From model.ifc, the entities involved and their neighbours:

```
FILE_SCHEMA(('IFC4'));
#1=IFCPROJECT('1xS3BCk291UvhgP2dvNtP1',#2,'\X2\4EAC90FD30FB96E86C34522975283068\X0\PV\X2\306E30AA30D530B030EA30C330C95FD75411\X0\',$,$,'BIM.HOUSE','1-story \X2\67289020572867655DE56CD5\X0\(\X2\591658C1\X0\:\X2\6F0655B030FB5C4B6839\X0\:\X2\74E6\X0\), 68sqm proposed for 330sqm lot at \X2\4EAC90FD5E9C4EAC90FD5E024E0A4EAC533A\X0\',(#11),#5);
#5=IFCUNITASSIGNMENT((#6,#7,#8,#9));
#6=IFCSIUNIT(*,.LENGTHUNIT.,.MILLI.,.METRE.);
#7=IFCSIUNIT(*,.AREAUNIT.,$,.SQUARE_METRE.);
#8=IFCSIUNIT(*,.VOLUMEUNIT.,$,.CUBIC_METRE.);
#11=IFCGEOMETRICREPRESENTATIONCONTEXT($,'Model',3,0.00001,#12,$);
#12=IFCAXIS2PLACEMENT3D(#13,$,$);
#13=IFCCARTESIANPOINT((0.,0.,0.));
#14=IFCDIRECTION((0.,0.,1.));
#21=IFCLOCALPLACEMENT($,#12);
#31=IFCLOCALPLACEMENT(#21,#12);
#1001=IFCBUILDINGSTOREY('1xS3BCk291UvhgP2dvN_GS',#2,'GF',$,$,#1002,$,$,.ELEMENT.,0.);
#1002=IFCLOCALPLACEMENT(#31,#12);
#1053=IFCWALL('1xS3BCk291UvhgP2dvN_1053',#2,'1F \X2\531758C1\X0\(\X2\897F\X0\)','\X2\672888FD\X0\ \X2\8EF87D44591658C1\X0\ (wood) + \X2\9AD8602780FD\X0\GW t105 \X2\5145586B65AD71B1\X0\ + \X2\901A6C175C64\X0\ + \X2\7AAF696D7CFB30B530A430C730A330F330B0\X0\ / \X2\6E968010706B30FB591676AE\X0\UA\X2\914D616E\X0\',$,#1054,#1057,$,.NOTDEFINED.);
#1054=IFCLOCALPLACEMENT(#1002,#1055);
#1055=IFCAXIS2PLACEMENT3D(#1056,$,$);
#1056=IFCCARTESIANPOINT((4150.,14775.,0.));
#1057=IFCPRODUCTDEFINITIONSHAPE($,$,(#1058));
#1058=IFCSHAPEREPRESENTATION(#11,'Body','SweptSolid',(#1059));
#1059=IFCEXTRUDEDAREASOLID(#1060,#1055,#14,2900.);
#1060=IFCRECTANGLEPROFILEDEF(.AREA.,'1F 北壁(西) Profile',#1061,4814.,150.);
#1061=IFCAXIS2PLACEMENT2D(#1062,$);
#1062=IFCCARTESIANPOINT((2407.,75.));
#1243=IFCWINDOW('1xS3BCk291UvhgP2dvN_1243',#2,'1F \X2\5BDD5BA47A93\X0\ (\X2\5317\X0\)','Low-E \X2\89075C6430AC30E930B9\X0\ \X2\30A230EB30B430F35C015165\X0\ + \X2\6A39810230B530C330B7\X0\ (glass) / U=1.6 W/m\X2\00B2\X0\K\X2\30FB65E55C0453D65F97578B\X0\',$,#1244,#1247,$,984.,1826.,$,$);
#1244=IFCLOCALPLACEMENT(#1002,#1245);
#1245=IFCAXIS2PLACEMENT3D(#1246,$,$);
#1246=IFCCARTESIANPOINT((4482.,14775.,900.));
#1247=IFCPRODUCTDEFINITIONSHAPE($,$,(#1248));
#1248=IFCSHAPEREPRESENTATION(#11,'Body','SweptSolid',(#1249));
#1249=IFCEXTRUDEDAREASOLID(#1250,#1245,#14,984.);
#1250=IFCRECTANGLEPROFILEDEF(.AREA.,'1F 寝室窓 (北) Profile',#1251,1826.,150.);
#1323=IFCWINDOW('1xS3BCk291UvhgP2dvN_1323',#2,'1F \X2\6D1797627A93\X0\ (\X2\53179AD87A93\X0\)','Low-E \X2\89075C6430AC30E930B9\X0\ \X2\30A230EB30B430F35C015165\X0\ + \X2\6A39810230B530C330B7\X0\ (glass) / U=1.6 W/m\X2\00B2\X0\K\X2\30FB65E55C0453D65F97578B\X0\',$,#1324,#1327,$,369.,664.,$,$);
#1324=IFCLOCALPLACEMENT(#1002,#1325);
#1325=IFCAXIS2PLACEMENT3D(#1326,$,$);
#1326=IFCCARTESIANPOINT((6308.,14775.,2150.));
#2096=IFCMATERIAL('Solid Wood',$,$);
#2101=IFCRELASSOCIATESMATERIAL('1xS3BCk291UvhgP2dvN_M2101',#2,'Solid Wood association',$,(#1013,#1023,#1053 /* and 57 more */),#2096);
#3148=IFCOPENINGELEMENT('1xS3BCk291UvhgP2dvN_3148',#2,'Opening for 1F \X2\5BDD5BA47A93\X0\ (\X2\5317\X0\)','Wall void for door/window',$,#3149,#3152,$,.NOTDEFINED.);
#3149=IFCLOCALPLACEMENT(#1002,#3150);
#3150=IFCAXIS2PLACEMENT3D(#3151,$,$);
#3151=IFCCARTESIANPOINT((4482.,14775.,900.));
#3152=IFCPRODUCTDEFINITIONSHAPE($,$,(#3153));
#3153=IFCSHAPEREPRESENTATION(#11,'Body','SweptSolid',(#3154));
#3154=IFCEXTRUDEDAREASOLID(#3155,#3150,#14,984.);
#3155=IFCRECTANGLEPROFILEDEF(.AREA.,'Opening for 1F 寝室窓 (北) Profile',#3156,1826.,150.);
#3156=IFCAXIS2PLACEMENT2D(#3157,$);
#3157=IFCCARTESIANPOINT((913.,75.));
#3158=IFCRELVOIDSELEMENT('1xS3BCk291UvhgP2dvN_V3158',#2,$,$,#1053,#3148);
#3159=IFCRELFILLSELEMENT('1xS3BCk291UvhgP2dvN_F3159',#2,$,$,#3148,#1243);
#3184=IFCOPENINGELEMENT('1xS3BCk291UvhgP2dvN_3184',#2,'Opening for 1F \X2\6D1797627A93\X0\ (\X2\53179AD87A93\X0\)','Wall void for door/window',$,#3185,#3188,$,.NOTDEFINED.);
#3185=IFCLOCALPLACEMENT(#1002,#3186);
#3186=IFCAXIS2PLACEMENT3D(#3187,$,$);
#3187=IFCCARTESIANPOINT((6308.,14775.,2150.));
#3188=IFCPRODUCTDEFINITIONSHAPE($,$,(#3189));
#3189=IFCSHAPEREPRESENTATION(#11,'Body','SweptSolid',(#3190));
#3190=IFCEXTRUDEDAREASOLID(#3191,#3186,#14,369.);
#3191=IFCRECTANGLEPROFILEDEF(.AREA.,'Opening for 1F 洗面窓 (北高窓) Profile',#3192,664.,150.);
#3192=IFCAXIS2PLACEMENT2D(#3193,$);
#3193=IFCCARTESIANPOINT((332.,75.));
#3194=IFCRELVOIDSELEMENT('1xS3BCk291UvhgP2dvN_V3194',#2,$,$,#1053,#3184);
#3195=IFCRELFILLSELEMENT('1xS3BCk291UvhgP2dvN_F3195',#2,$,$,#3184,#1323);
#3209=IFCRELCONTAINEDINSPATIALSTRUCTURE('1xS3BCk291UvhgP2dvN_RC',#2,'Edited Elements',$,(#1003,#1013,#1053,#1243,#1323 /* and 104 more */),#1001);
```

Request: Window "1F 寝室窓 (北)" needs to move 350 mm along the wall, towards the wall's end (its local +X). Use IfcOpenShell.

```python
import ifcopenshell
import ifcopenshell.api.geometry
import ifcopenshell.util.placement
import ifcopenshell.util.unit

model = ifcopenshell.open("model.ifc")
unit_scale = ifcopenshell.util.unit.calculate_unit_scale(model)

window = model.by_guid("1xS3BCk291UvhgP2dvN_1243")
opening = window.FillsVoids[0].RelatingOpeningElement
wall = opening.VoidsElements[0].RelatingBuildingElement

wall_matrix = ifcopenshell.util.placement.get_local_placement(wall.ObjectPlacement)
shift = wall_matrix[:3, 0] * 0.35 / unit_scale
before = ifcopenshell.util.placement.get_local_placement(window.ObjectPlacement)[:3, 3].copy()

# The window is not placed relative to its opening, so move both.
for product in (opening, window):
    matrix = ifcopenshell.util.placement.get_local_placement(product.ObjectPlacement)
    matrix[:3, 3] += shift
    ifcopenshell.api.geometry.edit_object_placement(model, product=product, matrix=matrix, is_si=False)

after = ifcopenshell.util.placement.get_local_placement(window.ObjectPlacement)[:3, 3]
print("window moved by", (after - before).round(3) + 0.0)

model.write("model-out.ifc")
```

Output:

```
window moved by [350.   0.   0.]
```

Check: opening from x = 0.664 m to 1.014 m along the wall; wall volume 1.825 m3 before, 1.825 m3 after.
